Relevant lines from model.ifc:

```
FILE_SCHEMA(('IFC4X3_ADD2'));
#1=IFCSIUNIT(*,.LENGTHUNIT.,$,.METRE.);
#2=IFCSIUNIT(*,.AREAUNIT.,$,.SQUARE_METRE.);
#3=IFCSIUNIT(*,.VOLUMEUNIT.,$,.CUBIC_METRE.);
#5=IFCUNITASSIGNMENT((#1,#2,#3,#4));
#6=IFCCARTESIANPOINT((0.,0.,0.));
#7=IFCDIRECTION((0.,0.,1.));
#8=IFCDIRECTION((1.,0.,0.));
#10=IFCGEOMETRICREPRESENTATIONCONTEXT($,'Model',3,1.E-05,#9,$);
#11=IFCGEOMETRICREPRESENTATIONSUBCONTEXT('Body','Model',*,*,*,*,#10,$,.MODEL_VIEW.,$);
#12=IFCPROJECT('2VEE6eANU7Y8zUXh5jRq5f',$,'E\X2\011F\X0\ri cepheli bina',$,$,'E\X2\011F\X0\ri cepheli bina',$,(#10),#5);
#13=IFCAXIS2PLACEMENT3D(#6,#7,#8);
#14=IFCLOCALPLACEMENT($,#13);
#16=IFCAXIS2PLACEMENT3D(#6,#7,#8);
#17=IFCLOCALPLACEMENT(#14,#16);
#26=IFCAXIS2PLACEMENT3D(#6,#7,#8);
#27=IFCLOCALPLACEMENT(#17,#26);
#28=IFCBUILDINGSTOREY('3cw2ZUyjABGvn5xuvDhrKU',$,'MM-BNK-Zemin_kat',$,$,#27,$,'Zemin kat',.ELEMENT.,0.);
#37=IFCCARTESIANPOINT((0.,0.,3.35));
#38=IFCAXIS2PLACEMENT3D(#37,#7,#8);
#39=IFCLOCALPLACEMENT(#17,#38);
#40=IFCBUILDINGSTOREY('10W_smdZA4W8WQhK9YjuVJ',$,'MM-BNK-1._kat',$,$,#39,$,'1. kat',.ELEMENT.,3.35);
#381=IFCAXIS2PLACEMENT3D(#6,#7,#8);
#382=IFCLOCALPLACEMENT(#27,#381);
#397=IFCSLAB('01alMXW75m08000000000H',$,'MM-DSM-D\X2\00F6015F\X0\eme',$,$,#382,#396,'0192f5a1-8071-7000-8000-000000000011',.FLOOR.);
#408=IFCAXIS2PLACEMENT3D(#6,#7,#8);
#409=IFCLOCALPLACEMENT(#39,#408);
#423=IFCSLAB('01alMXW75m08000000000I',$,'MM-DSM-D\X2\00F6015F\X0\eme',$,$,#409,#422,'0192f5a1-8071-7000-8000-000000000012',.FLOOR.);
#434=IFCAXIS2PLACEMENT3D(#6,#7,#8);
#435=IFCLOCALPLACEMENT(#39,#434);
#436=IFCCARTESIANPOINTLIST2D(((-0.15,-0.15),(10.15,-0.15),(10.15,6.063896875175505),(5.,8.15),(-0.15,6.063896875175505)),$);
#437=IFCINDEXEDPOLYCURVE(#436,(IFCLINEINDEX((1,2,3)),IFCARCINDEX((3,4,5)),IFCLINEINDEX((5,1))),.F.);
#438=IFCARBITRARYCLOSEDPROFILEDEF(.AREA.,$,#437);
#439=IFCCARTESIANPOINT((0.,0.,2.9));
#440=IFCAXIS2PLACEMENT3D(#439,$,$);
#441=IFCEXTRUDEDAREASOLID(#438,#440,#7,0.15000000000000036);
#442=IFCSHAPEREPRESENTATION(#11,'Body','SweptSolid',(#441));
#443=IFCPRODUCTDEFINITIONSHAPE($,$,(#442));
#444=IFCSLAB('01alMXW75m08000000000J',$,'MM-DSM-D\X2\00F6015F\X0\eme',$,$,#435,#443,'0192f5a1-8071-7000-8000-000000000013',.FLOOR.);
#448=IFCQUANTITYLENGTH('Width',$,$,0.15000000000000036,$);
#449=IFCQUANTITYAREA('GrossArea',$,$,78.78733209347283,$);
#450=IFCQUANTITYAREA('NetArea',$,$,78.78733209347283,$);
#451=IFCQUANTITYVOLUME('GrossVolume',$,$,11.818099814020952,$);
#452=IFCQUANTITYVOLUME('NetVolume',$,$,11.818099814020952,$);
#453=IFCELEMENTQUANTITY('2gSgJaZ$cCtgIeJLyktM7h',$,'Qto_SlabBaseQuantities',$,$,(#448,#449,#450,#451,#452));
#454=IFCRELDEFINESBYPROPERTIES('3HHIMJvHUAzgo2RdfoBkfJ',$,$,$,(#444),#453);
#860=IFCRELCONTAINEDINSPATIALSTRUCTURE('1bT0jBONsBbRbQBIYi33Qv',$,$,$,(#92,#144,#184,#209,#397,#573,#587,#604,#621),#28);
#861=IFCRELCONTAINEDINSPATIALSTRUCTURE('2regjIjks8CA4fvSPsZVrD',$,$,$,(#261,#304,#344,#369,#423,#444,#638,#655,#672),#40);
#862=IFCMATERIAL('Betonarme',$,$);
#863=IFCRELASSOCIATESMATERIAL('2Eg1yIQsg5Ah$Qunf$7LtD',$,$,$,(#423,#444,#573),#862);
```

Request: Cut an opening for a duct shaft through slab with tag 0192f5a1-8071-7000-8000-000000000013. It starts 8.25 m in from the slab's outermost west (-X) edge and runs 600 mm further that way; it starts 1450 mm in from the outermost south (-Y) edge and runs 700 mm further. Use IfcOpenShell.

```python
import numpy as np
import ifcopenshell
import ifcopenshell.api.feature
import ifcopenshell.api.geometry
import ifcopenshell.api.pset
import ifcopenshell.api.root
import ifcopenshell.geom
import ifcopenshell.util.element
import ifcopenshell.util.placement
import ifcopenshell.util.representation
import ifcopenshell.util.shape
import ifcopenshell.util.unit

model = ifcopenshell.open("model.ifc")
unit_scale = ifcopenshell.util.unit.calculate_unit_scale(model)
area_scale = ifcopenshell.util.unit.calculate_unit_scale(model, "AREAUNIT")
volume_scale = ifcopenshell.util.unit.calculate_unit_scale(model, "VOLUMEUNIT")
settings = ifcopenshell.geom.settings()


def volume(element):
    """Net volume in cubic metres, openings subtracted."""
    shape = ifcopenshell.geom.create_shape(settings, element)
    return ifcopenshell.util.shape.get_volume(shape.geometry)


slab = model.by_guid("01alMXW75m08000000000J")
before = volume(slab)

# Extent in the slab's own axes, in metres. The edges named are its -X and -Y sides.
slab_shape = ifcopenshell.geom.create_shape(settings, slab)
vertices = ifcopenshell.util.shape.get_vertices(slab_shape.geometry)
x_min, y_min, bottom = vertices.min(axis=0)
top = vertices[:, 2].max()

opening = ifcopenshell.api.root.create_entity(model, ifc_class="IfcOpeningElement", name="Duct shaft opening", predefined_type="OPENING")
context = ifcopenshell.util.representation.get_context(model, "Model", "Body", "MODEL_VIEW")
width, depth = 0.6, 0.7
outline = [(0.0, 0.0), (width, 0.0), (width, depth), (0.0, depth), (0.0, 0.0)]
# Overshoot both faces by 50 mm so the cut is clean.
shape = ifcopenshell.api.geometry.add_slab_representation(
    model, context=context, depth=top - bottom + 0.1, polyline=outline
)
ifcopenshell.api.geometry.assign_representation(model, product=opening, representation=shape)

matrix = ifcopenshell.util.placement.get_local_placement(slab.ObjectPlacement)
matrix[:, 3] = matrix @ np.append(np.array([x_min + 8.25, y_min + 1.45, bottom - 0.05]) / unit_scale, 1.0)
ifcopenshell.api.geometry.edit_object_placement(model, product=opening, matrix=matrix, is_si=False)
ifcopenshell.api.feature.add_feature(model, feature=opening, element=slab)

after = volume(slab)

# Update the slab's stored quantities.
qto = model.by_id(ifcopenshell.util.element.get_pset(slab, "Qto_SlabBaseQuantities", should_inherit=False)["id"])
ifcopenshell.api.pset.edit_qto(model, qto=qto, properties={
    "NetArea": after / (top - bottom) / area_scale,
    "NetVolume": after / volume_scale,
})

print(f"slab volume {before:.3f} -> {after:.3f} m3")

model.write("model_rev.ifc")
```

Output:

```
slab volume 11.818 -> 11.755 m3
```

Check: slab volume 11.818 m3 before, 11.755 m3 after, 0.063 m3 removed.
